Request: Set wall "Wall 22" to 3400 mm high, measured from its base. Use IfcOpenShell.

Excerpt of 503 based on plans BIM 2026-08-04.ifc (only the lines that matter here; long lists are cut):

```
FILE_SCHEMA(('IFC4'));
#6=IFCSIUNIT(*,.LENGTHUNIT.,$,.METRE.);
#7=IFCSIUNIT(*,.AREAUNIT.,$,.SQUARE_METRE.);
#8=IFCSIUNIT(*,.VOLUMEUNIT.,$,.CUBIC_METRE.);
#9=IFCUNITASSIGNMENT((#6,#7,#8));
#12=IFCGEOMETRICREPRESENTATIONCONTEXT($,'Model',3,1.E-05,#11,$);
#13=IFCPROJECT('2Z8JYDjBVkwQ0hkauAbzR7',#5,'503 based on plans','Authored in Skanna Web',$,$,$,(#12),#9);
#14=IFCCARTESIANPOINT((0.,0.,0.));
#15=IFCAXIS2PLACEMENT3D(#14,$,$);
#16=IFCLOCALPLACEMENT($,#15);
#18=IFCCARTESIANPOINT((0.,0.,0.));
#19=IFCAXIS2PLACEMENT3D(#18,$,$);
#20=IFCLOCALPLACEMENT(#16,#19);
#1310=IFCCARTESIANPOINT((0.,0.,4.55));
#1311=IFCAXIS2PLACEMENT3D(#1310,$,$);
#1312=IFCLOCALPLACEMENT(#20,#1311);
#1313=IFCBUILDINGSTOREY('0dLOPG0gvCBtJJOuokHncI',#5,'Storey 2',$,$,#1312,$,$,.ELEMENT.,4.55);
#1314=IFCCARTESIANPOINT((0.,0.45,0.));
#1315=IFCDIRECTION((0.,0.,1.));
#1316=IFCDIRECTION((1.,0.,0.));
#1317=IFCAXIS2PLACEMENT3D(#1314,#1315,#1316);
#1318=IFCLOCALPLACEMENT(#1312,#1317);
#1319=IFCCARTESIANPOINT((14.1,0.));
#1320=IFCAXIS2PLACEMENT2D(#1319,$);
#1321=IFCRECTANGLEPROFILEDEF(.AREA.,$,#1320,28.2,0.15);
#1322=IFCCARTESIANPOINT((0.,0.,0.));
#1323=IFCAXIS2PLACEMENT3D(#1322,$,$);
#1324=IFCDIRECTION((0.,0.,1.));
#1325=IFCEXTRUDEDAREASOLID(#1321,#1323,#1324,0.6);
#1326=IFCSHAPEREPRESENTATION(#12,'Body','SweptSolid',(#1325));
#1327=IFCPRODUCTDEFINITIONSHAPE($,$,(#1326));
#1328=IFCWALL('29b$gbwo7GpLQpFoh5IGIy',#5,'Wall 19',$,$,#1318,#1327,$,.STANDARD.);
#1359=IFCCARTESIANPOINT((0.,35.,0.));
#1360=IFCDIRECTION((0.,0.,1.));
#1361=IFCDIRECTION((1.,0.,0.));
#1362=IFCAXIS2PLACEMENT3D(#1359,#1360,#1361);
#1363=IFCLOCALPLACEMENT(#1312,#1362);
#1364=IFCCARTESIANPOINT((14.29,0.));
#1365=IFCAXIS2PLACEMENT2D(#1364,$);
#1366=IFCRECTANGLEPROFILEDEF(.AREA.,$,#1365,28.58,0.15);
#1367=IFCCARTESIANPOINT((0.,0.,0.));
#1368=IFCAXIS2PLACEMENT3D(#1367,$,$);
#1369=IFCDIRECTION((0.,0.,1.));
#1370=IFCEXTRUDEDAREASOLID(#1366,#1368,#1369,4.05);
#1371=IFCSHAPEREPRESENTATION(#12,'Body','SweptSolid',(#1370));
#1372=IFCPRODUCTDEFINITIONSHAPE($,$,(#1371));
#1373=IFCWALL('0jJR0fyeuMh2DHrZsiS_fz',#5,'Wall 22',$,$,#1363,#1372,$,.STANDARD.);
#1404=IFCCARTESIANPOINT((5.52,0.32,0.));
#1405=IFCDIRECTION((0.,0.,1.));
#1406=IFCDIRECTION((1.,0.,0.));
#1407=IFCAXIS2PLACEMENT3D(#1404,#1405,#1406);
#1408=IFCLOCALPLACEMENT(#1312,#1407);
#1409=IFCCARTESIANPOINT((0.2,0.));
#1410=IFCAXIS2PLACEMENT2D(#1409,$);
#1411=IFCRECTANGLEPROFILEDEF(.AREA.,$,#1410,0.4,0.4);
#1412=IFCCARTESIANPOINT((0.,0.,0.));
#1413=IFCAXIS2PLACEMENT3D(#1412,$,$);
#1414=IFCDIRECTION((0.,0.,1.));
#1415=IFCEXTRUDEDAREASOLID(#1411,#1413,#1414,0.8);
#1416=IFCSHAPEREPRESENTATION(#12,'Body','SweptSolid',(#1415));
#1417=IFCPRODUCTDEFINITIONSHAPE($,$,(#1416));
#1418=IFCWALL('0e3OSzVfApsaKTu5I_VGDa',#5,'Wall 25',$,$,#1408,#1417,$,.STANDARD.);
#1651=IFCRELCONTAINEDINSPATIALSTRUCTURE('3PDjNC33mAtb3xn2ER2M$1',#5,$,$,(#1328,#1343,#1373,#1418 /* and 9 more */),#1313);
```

```python
import ifcopenshell
import ifcopenshell.geom
import ifcopenshell.util.shape
import ifcopenshell.util.unit

model = ifcopenshell.open("503 based on plans BIM 2026-08-04.ifc")
unit_scale = ifcopenshell.util.unit.calculate_unit_scale(model)
settings = ifcopenshell.geom.settings()


def volume(element):
    """Net volume in cubic metres, openings subtracted."""
    shape = ifcopenshell.geom.create_shape(settings, element)
    return ifcopenshell.util.shape.get_volume(shape.geometry)


wall = model.by_guid("0jJR0fyeuMh2DHrZsiS_fz")
before = volume(wall)

body = next(r for r in wall.Representation.Representations if r.RepresentationIdentifier == "Body")
solid = body.Items[0]
old_height = solid.Depth
solid.Depth = 3.4 / unit_scale
after = volume(wall)

print(f"height {old_height:g} -> {solid.Depth:g}, volume {before:.3f} -> {after:.3f} m3")

model.write("503 based on plans BIM 2026-08-04_v2.ifc")
```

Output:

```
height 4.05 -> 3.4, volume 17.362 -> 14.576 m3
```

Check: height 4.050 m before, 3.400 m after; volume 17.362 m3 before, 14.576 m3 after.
